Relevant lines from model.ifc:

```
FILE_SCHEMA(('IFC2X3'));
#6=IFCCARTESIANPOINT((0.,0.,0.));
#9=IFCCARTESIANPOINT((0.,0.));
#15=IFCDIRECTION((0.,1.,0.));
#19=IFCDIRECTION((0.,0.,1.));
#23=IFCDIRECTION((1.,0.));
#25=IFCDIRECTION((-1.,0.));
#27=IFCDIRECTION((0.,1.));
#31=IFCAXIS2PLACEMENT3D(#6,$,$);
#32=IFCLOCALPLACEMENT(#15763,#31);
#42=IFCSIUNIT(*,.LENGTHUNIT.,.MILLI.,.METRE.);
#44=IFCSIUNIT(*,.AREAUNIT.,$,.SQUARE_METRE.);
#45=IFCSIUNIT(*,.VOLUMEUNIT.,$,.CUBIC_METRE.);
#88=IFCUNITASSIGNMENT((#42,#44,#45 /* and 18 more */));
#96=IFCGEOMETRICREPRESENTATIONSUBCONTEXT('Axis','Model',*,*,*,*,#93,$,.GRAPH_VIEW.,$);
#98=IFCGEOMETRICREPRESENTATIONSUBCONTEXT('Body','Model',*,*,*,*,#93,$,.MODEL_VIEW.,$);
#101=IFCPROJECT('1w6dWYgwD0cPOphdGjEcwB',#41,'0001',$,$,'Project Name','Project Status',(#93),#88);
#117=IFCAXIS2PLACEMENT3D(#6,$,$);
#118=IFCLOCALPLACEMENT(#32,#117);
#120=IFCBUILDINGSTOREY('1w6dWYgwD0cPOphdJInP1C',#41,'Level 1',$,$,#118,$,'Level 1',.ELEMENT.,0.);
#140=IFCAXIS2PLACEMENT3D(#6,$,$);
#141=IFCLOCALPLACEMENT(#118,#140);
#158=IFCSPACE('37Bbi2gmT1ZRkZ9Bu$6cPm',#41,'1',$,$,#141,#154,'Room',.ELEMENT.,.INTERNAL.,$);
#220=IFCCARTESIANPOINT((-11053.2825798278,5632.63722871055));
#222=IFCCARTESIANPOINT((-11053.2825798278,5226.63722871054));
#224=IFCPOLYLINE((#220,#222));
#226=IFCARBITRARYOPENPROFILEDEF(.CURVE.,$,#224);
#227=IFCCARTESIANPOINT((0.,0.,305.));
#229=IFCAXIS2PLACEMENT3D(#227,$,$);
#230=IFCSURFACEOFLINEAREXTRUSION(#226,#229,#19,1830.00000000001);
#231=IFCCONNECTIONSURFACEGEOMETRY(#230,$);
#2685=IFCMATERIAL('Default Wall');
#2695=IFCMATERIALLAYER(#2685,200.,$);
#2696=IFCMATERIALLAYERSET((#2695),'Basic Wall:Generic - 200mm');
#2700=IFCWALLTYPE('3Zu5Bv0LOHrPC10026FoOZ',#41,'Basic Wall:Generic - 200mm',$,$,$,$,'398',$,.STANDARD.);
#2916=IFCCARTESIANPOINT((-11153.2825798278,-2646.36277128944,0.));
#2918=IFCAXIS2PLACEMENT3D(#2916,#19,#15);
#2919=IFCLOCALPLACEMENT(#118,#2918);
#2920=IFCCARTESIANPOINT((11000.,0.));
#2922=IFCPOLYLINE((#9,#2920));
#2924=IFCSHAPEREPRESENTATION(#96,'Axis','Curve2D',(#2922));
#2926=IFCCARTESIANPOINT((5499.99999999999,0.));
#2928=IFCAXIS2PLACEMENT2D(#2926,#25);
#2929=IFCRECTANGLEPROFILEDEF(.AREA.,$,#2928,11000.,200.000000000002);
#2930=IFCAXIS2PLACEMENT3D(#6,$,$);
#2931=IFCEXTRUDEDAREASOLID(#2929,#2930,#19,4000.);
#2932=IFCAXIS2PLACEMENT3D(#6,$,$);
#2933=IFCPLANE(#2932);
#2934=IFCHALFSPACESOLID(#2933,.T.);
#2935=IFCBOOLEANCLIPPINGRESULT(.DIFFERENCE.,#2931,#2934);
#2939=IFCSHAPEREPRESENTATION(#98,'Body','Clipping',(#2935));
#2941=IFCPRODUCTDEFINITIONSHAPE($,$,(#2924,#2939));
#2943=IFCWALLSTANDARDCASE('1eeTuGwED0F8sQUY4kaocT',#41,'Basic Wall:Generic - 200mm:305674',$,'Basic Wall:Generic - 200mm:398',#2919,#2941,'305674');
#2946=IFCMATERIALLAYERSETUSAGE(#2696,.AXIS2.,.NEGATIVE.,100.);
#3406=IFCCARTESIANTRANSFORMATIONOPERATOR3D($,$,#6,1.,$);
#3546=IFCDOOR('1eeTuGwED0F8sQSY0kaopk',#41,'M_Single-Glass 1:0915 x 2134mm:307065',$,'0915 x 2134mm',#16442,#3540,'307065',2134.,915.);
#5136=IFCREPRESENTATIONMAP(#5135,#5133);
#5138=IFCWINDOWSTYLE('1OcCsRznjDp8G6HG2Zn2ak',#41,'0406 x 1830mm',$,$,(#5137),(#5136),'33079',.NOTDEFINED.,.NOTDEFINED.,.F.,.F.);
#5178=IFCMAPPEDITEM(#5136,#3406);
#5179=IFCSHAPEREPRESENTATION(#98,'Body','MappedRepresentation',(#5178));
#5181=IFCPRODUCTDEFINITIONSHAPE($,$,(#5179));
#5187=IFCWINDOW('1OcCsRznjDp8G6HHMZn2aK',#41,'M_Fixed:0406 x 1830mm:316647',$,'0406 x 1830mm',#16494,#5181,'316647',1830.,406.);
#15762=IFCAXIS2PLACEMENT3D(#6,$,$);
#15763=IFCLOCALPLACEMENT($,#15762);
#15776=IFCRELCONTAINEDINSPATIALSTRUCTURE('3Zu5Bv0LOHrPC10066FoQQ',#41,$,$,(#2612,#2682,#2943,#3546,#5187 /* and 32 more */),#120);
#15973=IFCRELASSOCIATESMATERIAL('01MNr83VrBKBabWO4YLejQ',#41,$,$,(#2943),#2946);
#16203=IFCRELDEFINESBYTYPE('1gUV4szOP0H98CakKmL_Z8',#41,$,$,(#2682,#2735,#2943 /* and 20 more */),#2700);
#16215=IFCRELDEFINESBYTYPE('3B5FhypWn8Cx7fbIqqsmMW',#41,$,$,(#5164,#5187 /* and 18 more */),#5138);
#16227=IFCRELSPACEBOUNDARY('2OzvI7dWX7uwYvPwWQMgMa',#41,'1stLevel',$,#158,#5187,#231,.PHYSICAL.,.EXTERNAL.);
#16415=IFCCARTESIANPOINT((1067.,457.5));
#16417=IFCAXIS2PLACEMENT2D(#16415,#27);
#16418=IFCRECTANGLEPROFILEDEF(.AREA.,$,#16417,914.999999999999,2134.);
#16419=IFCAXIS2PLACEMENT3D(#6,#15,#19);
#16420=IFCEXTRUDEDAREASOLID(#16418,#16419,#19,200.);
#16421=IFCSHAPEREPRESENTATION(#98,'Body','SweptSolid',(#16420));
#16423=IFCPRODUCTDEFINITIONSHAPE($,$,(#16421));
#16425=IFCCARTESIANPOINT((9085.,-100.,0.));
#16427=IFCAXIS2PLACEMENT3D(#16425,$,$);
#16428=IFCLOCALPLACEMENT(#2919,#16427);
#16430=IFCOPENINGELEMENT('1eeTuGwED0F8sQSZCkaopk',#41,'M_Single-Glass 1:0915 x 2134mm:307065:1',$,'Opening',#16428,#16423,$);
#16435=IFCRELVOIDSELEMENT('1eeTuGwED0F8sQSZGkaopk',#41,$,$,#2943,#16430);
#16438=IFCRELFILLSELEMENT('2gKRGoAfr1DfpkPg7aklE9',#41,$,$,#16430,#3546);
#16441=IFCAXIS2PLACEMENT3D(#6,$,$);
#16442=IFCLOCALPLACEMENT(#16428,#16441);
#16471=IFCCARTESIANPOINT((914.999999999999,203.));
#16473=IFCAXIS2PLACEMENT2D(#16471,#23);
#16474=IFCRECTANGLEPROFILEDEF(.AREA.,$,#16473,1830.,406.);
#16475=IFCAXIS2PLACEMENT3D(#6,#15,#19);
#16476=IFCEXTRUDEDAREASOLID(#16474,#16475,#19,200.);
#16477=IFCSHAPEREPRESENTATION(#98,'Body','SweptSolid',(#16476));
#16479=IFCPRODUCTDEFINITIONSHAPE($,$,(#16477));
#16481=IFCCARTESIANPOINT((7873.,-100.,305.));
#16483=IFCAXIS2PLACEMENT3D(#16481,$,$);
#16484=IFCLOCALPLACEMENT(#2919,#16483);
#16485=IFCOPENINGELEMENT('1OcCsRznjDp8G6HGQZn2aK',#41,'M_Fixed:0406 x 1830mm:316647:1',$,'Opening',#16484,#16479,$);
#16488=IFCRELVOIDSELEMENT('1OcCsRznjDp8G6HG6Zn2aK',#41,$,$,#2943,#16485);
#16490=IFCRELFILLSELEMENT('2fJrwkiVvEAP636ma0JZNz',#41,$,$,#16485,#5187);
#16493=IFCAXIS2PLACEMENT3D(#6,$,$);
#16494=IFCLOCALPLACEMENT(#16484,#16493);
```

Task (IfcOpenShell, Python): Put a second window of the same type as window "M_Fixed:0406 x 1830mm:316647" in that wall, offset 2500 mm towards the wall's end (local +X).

```python
import numpy as np
import ifcopenshell
import ifcopenshell.api.feature
import ifcopenshell.api.geometry
import ifcopenshell.api.root
import ifcopenshell.geom
import ifcopenshell.util.element
import ifcopenshell.util.placement
import ifcopenshell.util.shape
import ifcopenshell.util.unit

model = ifcopenshell.open("model.ifc")
unit_scale = ifcopenshell.util.unit.calculate_unit_scale(model)
settings = ifcopenshell.geom.settings()


def volume(element):
    """Net volume in cubic metres, openings subtracted."""
    shape = ifcopenshell.geom.create_shape(settings, element)
    return ifcopenshell.util.shape.get_volume(shape.geometry)


def reuse_history(source, copy):
    """copy_class also copies each property set's owner history, people and application; keep the originals."""
    for rel in copy.IsDefinedBy:
        if rel.is_a("IfcRelDefinesByProperties") and (history := rel.RelatingPropertyDefinition.OwnerHistory):
            rel.RelatingPropertyDefinition.OwnerHistory = source.OwnerHistory
            ifcopenshell.util.element.remove_deep2(model, history)


window = model.by_id(5187)
opening = window.FillsVoids[0].RelatingOpeningElement
wall = opening.VoidsElements[0].RelatingBuildingElement
before = volume(wall)
shift = ifcopenshell.util.placement.get_local_placement(wall.ObjectPlacement)[:3, 0] * 2.5 / unit_scale

# copy_class copies the void relationship, type, container and properties, but no geometry.
new_opening = ifcopenshell.api.root.copy_class(model, product=opening)
new_opening.Representation = ifcopenshell.util.element.copy_deep(
    model, opening.Representation, exclude=["IfcGeometricRepresentationContext", "IfcRepresentationMap"]
)
new_opening.Name = "M_Fixed:0406 x 1830mm"
new_window = ifcopenshell.api.root.copy_class(model, product=window)
new_window.Representation = ifcopenshell.util.element.copy_deep(
    model, window.Representation, exclude=["IfcGeometricRepresentationContext", "IfcRepresentationMap"]
)
new_window.Name = "M_Fixed:0406 x 1830mm"
new_window.Tag = None
reuse_history(window, new_window)
fills = ifcopenshell.api.feature.add_filling(model, opening=new_opening, element=new_window)
fills.OwnerHistory = new_window.OwnerHistory  # required in IFC2X3

for old, new in ((opening, new_opening), (window, new_window)):
    matrix = ifcopenshell.util.placement.get_local_placement(old.ObjectPlacement)
    matrix[:3, 3] += shift
    ifcopenshell.api.geometry.edit_object_placement(model, product=new, matrix=matrix, is_si=False)

# The copied space boundaries still share their surfaces with the original.
for rel in new_window.ProvidesBoundaries:
    if rel.ConnectionGeometry:
        rel.ConnectionGeometry = ifcopenshell.util.element.copy_deep(model, rel.ConnectionGeometry)

# Space boundary surfaces are stored in each space's coordinates; move them too.
for rel in new_window.ProvidesBoundaries:
    if not rel.ConnectionGeometry:
        continue
    surface = rel.ConnectionGeometry.SurfaceOnRelatingElement
    space_matrix = ifcopenshell.util.placement.get_local_placement(rel.RelatingSpace.ObjectPlacement)
    point = np.array(surface.Position.Location.Coordinates) + space_matrix[:3, :3].T @ shift
    surface.Position = model.createIfcAxis2Placement3D(
        model.createIfcCartesianPoint(point.tolist()), surface.Position.Axis, surface.Position.RefDirection
    )

after = volume(wall)

print(f"wall volume {before:.3f} -> {after:.3f} m3")

model.write("model_edited.ifc")
```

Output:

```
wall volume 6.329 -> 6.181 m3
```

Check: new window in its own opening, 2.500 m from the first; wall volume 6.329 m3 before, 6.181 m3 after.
